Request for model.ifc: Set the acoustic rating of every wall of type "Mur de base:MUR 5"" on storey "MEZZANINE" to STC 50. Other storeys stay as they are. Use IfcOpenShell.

First a look at what the model holds.

```python
import ifcopenshell
import ifcopenshell.util.element

model = ifcopenshell.open("model.ifc")
print(model.schema)
storey = next(s for s in model.by_type("IfcBuildingStorey") if s.Name == "MEZZANINE")
walls = [e for e in ifcopenshell.util.element.get_decomposition(storey) if e.is_a("IfcWall")]
seen = {}
for e in walls:
    element_type = ifcopenshell.util.element.get_type(e)
    key = (element_type.Name if element_type != e and element_type else None, ifcopenshell.util.element.get_pset(e, "Pset_WallCommon", "AcousticRating"))
    seen[key] = seen.get(key, 0) + 1
for (name, value), count in sorted(seen.items(), key=str):
    print(count, "x", name, "|", value)
```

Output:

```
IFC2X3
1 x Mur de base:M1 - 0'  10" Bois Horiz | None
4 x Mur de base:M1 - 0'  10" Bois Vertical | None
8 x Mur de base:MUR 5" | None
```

```python
import ifcopenshell
import ifcopenshell.api.pset
import ifcopenshell.util.element

model = ifcopenshell.open("model.ifc")

storey = next(s for s in model.by_type("IfcBuildingStorey") if s.Name == "MEZZANINE")
walls = [e for e in ifcopenshell.util.element.get_decomposition(storey) if e.is_a("IfcWall")]

count = 0
for e in walls:
    element_type = ifcopenshell.util.element.get_type(e)
    if element_type in (None, e) or element_type.Name != 'Mur de base:MUR 5"':
        continue
    # add_pset returns the element's existing set when there is one.
    pset = ifcopenshell.api.pset.add_pset(model, product=e, name="Pset_WallCommon")
    ifcopenshell.api.pset.edit_pset(model, pset=pset, properties={"AcousticRating": "STC 50"})
    count += 1

print(count, "walls updated")

model.write("model_v2.ifc")
```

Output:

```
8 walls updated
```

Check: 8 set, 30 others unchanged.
